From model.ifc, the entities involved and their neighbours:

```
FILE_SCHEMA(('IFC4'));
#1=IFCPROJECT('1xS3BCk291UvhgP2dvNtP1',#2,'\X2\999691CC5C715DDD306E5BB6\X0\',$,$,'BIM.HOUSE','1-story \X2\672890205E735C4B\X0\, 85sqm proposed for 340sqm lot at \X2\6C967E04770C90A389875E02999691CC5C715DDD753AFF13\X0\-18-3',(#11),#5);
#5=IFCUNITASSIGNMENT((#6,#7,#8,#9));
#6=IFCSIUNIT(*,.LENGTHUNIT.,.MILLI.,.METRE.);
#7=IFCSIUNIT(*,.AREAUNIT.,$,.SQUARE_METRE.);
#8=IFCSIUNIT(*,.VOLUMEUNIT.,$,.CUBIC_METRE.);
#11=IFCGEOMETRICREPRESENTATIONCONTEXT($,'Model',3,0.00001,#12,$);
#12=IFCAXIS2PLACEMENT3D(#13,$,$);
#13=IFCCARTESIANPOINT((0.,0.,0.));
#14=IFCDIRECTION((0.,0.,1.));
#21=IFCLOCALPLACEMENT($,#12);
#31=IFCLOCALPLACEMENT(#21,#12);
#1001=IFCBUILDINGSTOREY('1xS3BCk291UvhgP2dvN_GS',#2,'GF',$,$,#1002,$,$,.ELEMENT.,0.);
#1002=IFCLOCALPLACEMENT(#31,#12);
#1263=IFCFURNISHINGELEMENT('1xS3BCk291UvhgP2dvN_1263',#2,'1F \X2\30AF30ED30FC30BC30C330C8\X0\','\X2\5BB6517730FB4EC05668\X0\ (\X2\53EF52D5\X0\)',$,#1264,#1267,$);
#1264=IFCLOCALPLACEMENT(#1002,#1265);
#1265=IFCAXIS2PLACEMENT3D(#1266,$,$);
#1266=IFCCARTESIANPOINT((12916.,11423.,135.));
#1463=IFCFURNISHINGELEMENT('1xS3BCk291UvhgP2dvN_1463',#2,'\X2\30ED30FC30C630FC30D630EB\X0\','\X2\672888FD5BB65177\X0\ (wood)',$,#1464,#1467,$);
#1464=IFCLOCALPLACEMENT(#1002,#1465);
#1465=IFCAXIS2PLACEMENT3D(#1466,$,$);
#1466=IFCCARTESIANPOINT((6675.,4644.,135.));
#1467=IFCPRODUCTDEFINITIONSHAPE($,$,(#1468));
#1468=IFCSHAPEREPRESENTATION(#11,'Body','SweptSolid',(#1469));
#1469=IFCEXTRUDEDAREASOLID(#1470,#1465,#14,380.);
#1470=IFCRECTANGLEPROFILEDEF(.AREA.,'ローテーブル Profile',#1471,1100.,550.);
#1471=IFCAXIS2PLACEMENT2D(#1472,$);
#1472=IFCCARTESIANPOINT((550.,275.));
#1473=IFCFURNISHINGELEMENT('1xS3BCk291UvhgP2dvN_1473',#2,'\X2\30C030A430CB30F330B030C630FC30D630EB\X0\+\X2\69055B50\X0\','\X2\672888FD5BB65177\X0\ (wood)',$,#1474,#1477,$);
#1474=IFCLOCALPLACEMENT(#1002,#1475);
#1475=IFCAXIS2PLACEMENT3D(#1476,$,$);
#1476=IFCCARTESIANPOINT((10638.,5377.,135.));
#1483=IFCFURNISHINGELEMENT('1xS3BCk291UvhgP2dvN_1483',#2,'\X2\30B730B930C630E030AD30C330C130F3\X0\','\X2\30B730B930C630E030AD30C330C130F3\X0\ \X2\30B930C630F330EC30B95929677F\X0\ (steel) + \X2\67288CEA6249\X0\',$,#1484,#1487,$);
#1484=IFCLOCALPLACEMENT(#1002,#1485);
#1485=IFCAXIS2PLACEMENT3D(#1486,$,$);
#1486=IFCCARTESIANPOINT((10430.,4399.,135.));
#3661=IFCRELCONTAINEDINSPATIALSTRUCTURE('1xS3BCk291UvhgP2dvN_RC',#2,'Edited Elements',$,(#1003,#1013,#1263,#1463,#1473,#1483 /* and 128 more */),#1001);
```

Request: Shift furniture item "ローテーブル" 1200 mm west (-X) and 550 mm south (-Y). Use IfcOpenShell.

```python
import ifcopenshell
import ifcopenshell.api.geometry
import ifcopenshell.util.placement
import ifcopenshell.util.unit

model = ifcopenshell.open("model.ifc")
unit_scale = ifcopenshell.util.unit.calculate_unit_scale(model)

item = model.by_guid("1xS3BCk291UvhgP2dvN_1463")
matrix = ifcopenshell.util.placement.get_local_placement(item.ObjectPlacement)
matrix[0, 3] -= 1.2 / unit_scale
matrix[1, 3] -= 0.55 / unit_scale
ifcopenshell.api.geometry.edit_object_placement(model, product=item, matrix=matrix, is_si=False)

print(ifcopenshell.util.placement.get_local_placement(item.ObjectPlacement).round(3) + 0.0)

model.write("model_updated.ifc")
```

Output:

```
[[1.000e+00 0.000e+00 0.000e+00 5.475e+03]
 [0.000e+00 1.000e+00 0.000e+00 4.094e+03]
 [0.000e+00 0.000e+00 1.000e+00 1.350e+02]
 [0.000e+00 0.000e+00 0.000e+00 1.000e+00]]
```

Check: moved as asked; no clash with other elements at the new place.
